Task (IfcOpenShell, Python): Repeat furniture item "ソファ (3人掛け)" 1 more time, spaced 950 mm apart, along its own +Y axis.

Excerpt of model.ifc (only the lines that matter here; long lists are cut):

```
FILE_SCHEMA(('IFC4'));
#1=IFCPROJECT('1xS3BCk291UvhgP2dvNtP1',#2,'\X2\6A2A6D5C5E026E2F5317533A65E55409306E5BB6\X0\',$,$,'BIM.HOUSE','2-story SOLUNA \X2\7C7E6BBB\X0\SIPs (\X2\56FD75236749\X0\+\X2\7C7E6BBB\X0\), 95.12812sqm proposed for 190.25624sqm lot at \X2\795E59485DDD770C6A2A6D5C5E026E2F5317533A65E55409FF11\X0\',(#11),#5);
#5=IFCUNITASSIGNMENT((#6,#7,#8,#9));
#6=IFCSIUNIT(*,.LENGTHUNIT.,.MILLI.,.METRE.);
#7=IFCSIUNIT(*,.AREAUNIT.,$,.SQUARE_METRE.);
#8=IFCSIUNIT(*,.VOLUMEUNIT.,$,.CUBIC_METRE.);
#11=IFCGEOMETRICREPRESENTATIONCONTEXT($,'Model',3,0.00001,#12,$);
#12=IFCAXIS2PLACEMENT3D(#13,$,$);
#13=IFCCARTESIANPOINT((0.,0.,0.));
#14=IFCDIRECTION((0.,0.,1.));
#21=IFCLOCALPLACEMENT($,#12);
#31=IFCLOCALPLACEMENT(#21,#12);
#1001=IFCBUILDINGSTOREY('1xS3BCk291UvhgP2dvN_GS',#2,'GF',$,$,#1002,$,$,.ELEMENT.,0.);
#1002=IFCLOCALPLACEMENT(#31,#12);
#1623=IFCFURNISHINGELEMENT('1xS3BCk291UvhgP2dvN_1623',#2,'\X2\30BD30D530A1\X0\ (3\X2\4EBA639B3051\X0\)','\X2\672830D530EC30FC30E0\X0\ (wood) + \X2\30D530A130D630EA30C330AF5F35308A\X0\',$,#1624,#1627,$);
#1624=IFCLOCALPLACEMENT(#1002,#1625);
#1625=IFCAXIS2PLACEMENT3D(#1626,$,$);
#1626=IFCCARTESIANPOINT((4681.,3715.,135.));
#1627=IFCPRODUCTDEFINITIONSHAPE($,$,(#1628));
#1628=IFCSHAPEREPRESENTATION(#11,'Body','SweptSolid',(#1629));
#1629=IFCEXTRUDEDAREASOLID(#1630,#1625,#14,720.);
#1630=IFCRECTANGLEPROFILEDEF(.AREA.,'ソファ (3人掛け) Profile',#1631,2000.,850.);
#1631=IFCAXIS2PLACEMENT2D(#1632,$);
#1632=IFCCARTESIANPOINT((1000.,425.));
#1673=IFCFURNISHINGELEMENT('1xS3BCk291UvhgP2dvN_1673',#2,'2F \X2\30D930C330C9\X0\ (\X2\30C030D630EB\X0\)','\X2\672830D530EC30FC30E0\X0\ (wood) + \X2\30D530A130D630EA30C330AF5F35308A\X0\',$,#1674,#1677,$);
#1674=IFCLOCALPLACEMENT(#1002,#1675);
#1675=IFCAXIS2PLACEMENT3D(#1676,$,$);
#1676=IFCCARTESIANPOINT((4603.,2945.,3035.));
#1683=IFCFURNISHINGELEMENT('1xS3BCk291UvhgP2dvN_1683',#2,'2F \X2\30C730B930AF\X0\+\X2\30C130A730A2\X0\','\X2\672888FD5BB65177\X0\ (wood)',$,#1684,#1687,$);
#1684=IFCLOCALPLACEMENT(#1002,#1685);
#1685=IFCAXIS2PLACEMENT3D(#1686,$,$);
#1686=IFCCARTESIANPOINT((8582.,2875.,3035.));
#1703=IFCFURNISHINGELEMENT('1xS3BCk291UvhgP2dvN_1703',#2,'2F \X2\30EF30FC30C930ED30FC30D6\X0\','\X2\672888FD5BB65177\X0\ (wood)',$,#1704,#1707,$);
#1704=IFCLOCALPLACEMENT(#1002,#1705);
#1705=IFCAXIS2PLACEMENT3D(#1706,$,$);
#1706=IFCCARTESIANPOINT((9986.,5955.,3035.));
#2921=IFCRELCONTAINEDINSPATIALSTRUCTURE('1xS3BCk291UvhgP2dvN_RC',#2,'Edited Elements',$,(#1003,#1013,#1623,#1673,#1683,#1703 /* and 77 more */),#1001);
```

```python
import ifcopenshell
import ifcopenshell.api.geometry
import ifcopenshell.api.root
import ifcopenshell.util.element
import ifcopenshell.util.placement

model = ifcopenshell.open("model.ifc")


def reuse_history(source, copy):
    """copy_class also copies each property set's owner history, people and application; keep the originals."""
    for rel in copy.IsDefinedBy:
        if rel.is_a("IfcRelDefinesByProperties") and (history := rel.RelatingPropertyDefinition.OwnerHistory):
            rel.RelatingPropertyDefinition.OwnerHistory = source.OwnerHistory
            ifcopenshell.util.element.remove_deep2(model, history)


source = model.by_id(1623)
base = ifcopenshell.util.placement.get_local_placement(source.ObjectPlacement)
step = base[:3, 1] * 950.0

for i in range(1, 2):
    copy = ifcopenshell.api.root.copy_class(model, product=source)
    copy.Representation = ifcopenshell.util.element.copy_deep(
        model, source.Representation, exclude=["IfcGeometricRepresentationContext", "IfcRepresentationMap"]
    )
    reuse_history(source, copy)
    matrix = base.copy()
    matrix[:3, 3] += i * step
    print("added at", matrix[:3, 3].round(3) + 0.0)
    ifcopenshell.api.geometry.edit_object_placement(model, product=copy, matrix=matrix, is_si=False)

model.write("model-out.ifc")
```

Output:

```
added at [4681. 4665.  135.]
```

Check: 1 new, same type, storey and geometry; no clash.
